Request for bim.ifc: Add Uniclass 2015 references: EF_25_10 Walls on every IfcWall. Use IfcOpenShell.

First a look at what the model holds.

```python
import ifcopenshell

model = ifcopenshell.open("bim.ifc")
print(model.schema)
print("classifications:", [c.Name for c in model.by_type("IfcClassification")])
for ifc_class in ("IfcDoor", "IfcRoof", "IfcStair", "IfcWall", "IfcWindow"):
    print(ifc_class, len(model.by_type(ifc_class)))
```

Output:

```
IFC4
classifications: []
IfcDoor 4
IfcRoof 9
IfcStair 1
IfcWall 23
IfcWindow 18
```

```python
import ifcopenshell
import ifcopenshell.api.classification

model = ifcopenshell.open("bim.ifc")

system = ifcopenshell.api.classification.add_classification(model, classification="Uniclass 2015")

codes = {
    "IfcWall": ("EF_25_10", "Walls"),
}
for ifc_class, (code, name) in codes.items():
    products = model.by_type(ifc_class)
    ifcopenshell.api.classification.add_reference(
        model, products=products, classification=system, identification=code, name=name
    )
    print(code, len(products))

model.write("bim_updated.ifc")
```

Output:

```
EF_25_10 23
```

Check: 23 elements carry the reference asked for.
